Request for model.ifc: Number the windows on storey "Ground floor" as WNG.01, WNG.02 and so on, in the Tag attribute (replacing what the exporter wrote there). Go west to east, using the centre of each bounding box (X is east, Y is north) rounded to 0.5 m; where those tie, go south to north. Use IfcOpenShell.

First a look at what the model holds.

```python
import ifcopenshell
import ifcopenshell.util.element
import ifcopenshell.util.placement

model = ifcopenshell.open("model.ifc")
print(model.schema)
storey = next(s for s in model.by_type("IfcBuildingStorey") if s.Name == "Ground floor")
windows = [e for e in ifcopenshell.util.element.get_decomposition(storey) if e.is_a("IfcWindow")]
for e in sorted(windows, key=lambda e: e.id()):
    origin = ifcopenshell.util.placement.get_local_placement(e.ObjectPlacement)[:3, 3]
    print(e.id(), e.Tag, e.Name, origin.round(2) + 0.0, sep=" | ")
```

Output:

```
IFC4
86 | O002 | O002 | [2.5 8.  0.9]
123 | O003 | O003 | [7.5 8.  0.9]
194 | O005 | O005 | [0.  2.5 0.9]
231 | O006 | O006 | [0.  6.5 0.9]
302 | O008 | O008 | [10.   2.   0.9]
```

```python
import ifcopenshell
import ifcopenshell.geom
import ifcopenshell.util.element
import ifcopenshell.util.shape

model = ifcopenshell.open("model.ifc")
settings = ifcopenshell.geom.settings()
settings.set("use-world-coords", True)


def centre(element):
    shape = ifcopenshell.geom.create_shape(settings, element)
    return ifcopenshell.util.shape.get_bbox_centroid(shape.geometry)


storey = next(s for s in model.by_type("IfcBuildingStorey") if s.Name == "Ground floor")
windows = [e for e in ifcopenshell.util.element.get_decomposition(storey) if e.is_a("IfcWindow")]

# Insertion points can sit at a corner or the storey origin, so sort by the geometry (in metres).
centres = {e: centre(e) for e in windows}
windows.sort(key=lambda e: (round(centres[e][0] / 0.5), centres[e][1]))

for i, e in enumerate(windows, start=1):
    number = f"WNG.{i:02d}"
    e.Tag = number
    print(e.id(), number)

model.write("model_rev.ifc")
```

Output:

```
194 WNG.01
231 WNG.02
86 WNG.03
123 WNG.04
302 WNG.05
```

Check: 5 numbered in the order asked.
